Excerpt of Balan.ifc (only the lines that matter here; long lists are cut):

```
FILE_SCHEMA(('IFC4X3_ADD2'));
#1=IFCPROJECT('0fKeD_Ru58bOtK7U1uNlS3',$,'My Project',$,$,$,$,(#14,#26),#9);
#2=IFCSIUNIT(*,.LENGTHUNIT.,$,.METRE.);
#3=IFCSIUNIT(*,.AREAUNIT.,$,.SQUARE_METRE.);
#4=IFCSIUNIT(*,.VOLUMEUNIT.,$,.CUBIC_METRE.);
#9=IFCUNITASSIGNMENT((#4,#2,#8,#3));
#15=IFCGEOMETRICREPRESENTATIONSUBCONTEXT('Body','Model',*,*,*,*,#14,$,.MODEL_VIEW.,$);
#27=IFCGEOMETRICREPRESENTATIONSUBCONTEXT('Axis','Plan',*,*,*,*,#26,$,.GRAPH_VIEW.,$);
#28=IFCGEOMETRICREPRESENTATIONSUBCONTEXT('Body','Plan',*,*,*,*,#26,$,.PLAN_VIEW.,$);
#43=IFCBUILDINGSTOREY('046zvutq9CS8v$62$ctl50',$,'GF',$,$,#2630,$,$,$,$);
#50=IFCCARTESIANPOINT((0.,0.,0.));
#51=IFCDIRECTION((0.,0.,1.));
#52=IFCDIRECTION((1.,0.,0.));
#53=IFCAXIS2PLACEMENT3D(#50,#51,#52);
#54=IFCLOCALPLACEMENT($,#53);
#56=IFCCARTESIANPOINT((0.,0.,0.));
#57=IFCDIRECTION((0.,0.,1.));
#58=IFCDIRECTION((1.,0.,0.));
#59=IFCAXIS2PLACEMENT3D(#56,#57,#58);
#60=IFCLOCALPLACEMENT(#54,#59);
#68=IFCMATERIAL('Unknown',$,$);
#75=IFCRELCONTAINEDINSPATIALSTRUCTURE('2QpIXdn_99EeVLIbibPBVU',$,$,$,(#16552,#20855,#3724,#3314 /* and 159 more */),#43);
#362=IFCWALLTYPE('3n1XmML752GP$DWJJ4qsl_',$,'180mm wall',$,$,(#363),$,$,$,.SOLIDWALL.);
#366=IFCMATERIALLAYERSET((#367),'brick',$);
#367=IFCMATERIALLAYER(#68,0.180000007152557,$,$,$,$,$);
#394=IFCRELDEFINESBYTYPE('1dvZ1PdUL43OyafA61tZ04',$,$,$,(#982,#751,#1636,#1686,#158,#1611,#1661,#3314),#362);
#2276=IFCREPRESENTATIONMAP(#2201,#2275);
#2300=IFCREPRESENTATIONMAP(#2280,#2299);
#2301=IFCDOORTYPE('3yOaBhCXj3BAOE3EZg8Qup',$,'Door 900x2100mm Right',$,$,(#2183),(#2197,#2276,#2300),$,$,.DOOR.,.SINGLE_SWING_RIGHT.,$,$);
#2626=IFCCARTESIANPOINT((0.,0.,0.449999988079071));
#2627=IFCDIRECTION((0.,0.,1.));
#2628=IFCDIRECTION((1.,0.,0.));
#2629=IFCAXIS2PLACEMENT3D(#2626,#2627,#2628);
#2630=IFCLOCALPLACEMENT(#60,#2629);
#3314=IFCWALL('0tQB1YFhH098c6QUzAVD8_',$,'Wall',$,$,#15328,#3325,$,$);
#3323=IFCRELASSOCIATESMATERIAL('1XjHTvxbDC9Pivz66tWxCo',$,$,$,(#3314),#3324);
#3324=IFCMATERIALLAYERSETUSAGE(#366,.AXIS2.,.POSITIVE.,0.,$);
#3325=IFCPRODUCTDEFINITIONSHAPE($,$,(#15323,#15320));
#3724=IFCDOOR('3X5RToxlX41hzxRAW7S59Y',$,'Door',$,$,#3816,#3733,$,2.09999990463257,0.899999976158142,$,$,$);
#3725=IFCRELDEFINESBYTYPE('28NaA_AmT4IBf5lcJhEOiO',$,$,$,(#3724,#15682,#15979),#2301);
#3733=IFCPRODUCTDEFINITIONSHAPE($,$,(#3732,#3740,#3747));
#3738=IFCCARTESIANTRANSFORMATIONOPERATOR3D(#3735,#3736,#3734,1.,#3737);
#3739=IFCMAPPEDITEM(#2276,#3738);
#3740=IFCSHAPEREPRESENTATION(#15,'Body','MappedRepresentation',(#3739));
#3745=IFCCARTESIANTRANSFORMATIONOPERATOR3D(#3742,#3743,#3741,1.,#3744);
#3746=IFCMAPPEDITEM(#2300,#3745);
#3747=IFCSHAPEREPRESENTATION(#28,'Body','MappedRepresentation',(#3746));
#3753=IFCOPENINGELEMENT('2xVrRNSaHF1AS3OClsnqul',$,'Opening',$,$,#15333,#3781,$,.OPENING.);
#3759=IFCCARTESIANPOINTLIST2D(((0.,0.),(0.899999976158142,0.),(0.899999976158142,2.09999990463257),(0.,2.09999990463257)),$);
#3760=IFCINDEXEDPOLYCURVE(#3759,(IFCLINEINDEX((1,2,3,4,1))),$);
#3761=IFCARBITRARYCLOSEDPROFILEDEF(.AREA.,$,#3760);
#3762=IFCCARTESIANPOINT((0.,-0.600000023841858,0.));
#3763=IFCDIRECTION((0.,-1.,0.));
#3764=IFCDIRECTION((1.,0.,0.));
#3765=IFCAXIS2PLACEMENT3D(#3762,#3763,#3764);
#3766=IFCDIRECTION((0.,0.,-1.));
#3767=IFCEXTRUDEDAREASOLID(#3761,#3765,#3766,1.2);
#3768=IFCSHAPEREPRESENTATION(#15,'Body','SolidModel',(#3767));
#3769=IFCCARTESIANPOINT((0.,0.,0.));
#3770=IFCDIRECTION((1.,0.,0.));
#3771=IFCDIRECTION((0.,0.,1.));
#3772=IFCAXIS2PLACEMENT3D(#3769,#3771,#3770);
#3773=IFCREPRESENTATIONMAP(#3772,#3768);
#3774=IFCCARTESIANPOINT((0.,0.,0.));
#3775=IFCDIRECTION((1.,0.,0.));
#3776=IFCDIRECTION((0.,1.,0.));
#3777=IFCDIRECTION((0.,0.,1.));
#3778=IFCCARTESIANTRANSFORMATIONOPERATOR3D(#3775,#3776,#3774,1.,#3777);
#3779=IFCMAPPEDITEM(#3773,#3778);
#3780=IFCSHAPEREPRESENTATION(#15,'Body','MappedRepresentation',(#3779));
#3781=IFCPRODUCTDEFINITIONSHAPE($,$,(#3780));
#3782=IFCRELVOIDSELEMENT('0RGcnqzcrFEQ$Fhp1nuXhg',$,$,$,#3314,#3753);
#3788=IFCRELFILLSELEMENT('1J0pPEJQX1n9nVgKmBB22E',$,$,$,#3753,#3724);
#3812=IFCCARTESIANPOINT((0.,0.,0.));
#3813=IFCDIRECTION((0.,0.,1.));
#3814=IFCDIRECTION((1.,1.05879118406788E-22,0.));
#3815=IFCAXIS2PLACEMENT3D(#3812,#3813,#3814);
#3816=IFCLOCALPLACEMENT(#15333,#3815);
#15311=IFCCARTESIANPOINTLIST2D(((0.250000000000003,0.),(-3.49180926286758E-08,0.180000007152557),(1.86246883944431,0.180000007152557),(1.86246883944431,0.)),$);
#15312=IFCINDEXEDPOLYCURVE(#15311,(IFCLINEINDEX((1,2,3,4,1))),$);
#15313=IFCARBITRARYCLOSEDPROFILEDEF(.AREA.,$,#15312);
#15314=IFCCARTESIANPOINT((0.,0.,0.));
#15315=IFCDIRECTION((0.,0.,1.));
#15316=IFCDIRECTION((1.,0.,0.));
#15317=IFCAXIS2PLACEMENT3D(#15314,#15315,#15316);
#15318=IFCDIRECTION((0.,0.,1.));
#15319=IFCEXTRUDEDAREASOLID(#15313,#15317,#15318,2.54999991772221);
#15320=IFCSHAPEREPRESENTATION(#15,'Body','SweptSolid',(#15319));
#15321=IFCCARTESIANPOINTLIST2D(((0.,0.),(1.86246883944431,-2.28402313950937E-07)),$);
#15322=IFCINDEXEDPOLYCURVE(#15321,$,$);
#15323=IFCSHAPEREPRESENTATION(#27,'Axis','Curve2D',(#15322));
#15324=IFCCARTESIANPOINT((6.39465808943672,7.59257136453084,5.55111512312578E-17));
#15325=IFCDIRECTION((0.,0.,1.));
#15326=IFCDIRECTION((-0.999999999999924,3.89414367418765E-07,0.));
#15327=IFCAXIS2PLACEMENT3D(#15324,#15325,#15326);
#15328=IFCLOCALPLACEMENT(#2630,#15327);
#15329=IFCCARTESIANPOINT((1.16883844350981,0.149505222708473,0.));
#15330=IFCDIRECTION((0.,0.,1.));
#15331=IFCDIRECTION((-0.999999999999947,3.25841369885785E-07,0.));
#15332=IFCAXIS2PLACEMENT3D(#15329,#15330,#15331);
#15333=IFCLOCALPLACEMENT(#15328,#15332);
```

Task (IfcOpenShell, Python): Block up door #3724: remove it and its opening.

```python
import ifcopenshell
import ifcopenshell.api.feature
import ifcopenshell.api.root
import ifcopenshell.geom
import ifcopenshell.util.shape

model = ifcopenshell.open("Balan.ifc")
settings = ifcopenshell.geom.settings()


def volume(element):
    """Net volume in cubic metres, openings subtracted."""
    shape = ifcopenshell.geom.create_shape(settings, element)
    return ifcopenshell.util.shape.get_volume(shape.geometry)


door = model.by_id(3724)
opening = door.FillsVoids[0].RelatingOpeningElement
wall = opening.VoidsElements[0].RelatingBuildingElement
before = volume(wall)

ifcopenshell.api.root.remove_product(model, product=door)
ifcopenshell.api.feature.remove_feature(model, feature=opening)

after = volume(wall)

print(f"wall volume {before:.3f} -> {after:.3f} m3")

model.write("Balan-out.ifc")
```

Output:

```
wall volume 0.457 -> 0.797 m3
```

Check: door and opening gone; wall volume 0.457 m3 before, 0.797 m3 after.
